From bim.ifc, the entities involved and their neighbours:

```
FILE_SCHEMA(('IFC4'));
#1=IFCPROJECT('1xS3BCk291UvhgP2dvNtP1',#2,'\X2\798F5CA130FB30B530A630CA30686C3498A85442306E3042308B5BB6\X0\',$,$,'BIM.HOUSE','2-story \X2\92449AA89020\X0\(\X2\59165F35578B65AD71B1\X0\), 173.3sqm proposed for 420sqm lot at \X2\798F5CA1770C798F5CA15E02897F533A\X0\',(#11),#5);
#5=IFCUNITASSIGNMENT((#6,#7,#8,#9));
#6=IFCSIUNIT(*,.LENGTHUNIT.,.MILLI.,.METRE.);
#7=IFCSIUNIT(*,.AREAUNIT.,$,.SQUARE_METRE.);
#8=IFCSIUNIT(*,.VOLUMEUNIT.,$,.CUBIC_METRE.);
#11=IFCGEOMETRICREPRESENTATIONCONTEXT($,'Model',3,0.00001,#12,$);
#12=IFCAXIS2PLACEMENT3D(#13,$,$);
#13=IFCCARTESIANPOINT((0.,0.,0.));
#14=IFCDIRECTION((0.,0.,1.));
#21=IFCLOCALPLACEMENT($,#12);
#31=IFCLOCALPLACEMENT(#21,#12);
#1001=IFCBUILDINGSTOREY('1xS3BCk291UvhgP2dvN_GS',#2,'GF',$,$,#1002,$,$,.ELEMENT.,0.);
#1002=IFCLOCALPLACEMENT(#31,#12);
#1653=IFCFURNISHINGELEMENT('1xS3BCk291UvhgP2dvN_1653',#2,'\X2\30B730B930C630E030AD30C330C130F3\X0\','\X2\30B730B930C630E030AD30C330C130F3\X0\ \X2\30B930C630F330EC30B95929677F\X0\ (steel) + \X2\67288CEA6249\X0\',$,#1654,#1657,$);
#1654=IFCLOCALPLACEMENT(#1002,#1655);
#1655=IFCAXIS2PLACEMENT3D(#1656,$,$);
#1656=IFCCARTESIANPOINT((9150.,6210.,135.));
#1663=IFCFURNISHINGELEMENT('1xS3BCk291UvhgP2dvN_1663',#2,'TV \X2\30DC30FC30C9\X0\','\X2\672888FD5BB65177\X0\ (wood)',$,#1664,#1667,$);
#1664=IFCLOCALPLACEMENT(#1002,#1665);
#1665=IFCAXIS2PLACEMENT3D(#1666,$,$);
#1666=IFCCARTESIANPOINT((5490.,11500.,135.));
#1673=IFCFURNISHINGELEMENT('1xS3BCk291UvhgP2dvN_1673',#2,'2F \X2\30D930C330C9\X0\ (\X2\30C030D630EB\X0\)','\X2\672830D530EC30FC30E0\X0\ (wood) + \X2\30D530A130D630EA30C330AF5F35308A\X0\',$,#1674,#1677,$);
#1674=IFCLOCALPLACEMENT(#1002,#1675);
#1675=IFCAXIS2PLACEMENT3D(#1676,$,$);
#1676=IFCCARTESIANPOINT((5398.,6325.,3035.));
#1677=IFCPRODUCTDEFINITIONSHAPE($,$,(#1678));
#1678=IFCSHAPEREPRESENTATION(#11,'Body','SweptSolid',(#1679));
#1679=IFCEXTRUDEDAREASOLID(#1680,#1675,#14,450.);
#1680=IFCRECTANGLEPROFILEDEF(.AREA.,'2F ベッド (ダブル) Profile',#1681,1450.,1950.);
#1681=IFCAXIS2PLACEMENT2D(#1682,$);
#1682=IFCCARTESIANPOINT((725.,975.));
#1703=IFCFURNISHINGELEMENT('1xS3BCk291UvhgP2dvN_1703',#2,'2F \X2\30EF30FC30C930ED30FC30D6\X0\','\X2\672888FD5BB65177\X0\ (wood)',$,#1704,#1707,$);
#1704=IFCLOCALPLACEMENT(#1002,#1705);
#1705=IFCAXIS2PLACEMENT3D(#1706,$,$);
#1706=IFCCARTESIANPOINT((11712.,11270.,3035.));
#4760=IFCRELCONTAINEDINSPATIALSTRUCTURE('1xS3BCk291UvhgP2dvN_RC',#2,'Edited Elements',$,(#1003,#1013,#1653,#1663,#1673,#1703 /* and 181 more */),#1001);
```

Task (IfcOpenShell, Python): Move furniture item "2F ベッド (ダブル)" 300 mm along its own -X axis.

```python
import ifcopenshell
import ifcopenshell.api.geometry
import ifcopenshell.util.placement

model = ifcopenshell.open("bim.ifc")

item = model.by_id(1673)
matrix = ifcopenshell.util.placement.get_local_placement(item.ObjectPlacement)
matrix[:3, 3] -= matrix[:3, 0] * 300.0
ifcopenshell.api.geometry.edit_object_placement(model, product=item, matrix=matrix, is_si=False)

print(ifcopenshell.util.placement.get_local_placement(item.ObjectPlacement).round(3) + 0.0)

model.write("bim_updated.ifc")
```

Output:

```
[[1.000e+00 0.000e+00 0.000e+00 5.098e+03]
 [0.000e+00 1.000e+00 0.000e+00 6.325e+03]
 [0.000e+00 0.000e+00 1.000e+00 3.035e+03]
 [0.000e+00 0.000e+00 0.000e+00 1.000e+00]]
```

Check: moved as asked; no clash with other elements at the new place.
